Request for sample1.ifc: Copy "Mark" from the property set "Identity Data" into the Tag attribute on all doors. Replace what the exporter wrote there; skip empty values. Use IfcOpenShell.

First a look at what the model holds.

```python
import ifcopenshell
import ifcopenshell.util.element

model = ifcopenshell.open("sample1.ifc")
print(model.schema)
doors = model.by_type("IfcDoor")
print(len(doors), "doors")
for e in doors[:8]:
    source = ifcopenshell.util.element.get_pset(e, "Identity Data", "Mark")
    target = e.Tag
    print(e.id(), repr(source), repr(target), sep=" | ")
```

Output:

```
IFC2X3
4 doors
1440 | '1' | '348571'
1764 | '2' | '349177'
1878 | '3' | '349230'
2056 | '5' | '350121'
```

```python
import ifcopenshell
import ifcopenshell.util.element

model = ifcopenshell.open("sample1.ifc")

count = 0
for e in model.by_type("IfcDoor"):
    value = ifcopenshell.util.element.get_pset(e, "Identity Data", "Mark")
    current = e.Tag
    if not value or not value.strip() or current == value:
        continue
    e.Tag = value
    count += 1

print(count, "doors updated")

model.write("sample1_rev.ifc")
```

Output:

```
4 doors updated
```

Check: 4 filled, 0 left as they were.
